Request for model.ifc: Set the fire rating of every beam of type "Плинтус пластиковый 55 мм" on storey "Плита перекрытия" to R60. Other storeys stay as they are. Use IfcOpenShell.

First a look at what the model holds.

```python
import ifcopenshell
import ifcopenshell.util.element

model = ifcopenshell.open("model.ifc")
print(model.schema)
storey = next(s for s in model.by_type("IfcBuildingStorey") if s.Name == "Плита перекрытия")
beams = [e for e in ifcopenshell.util.element.get_decomposition(storey) if e.is_a("IfcBeam")]
seen = {}
for e in beams:
    element_type = ifcopenshell.util.element.get_type(e)
    key = (element_type.Name if element_type != e and element_type else None, ifcopenshell.util.element.get_pset(e, "Pset_BeamCommon", "FireRating"))
    seen[key] = seen.get(key, 0) + 1
for (name, value), count in sorted(seen.items(), key=str):
    print(count, "x", name, "|", value)
```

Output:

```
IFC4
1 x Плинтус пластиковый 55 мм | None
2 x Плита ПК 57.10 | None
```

```python
import ifcopenshell
import ifcopenshell.api.pset
import ifcopenshell.util.element

model = ifcopenshell.open("model.ifc")

storey = next(s for s in model.by_type("IfcBuildingStorey") if s.Name == "Плита перекрытия")
beams = [e for e in ifcopenshell.util.element.get_decomposition(storey) if e.is_a("IfcBeam")]

count = 0
for e in beams:
    element_type = ifcopenshell.util.element.get_type(e)
    if element_type in (None, e) or element_type.Name != "Плинтус пластиковый 55 мм":
        continue
    # add_pset returns the element's existing set when there is one.
    pset = ifcopenshell.api.pset.add_pset(model, product=e, name="Pset_BeamCommon")
    ifcopenshell.api.pset.edit_pset(model, pset=pset, properties={"FireRating": "R60"})
    count += 1

print(count, "beams updated")

model.write("model_edited.ifc")
```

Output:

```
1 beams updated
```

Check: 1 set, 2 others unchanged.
